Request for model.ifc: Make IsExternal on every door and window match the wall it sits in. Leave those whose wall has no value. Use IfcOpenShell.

First a look at what the model holds.

```python
import ifcopenshell
import ifcopenshell.util.element

model = ifcopenshell.open("model.ifc")
print(model.schema)
seen = {}
for e in model.by_type("IfcDoor") + model.by_type("IfcWindow"):
    if not e.FillsVoids:
        continue
    host = e.FillsVoids[0].RelatingOpeningElement.VoidsElements[0].RelatingBuildingElement
    own = ifcopenshell.util.element.get_pset(e, f"Pset_{e.is_a()[3:].removesuffix('StandardCase')}Common", "IsExternal")
    wall = ifcopenshell.util.element.get_pset(host, "Pset_WallCommon", "IsExternal")
    seen[e.is_a(), own, wall] = seen.get((e.is_a(), own, wall), 0) + 1
for (cls, own, wall), count in sorted(seen.items(), key=str):
    print(count, cls, "IsExternal:", own, "| host wall:", wall)
```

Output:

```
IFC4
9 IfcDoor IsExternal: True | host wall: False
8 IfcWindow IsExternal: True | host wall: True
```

```python
import ifcopenshell
import ifcopenshell.api.pset
import ifcopenshell.util.element

model = ifcopenshell.open("model.ifc")

count = 0
for ifc_class, pset_name in (("IfcDoor", "Pset_DoorCommon"), ("IfcWindow", "Pset_WindowCommon")):
    for e in model.by_type(ifc_class):
        if not e.FillsVoids:
            continue
        host = e.FillsVoids[0].RelatingOpeningElement.VoidsElements[0].RelatingBuildingElement
        external = ifcopenshell.util.element.get_pset(host, "Pset_WallCommon", "IsExternal")
        if external is None or ifcopenshell.util.element.get_pset(e, pset_name, "IsExternal") == external:
            continue
        pset = ifcopenshell.api.pset.add_pset(model, product=e, name=pset_name)
        ifcopenshell.api.pset.edit_pset(model, pset=pset, properties={"IsExternal": external})
        count += 1

print(count, "updated")

model.write("model_v2.ifc")
```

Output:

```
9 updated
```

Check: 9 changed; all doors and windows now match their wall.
